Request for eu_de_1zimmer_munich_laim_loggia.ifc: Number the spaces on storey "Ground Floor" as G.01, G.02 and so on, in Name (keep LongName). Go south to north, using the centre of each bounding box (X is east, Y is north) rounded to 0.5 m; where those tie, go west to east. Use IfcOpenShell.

First a look at what the model holds.

```python
import ifcopenshell
import ifcopenshell.util.element
import ifcopenshell.util.placement

model = ifcopenshell.open("eu_de_1zimmer_munich_laim_loggia.ifc")
print(model.schema)
storey = next(s for s in model.by_type("IfcBuildingStorey") if s.Name == "Ground Floor")
spaces = [e for e in ifcopenshell.util.element.get_decomposition(storey) if e.is_a("IfcSpace")]
for e in sorted(spaces, key=lambda e: e.id()):
    origin = ifcopenshell.util.placement.get_local_placement(e.ObjectPlacement)[:3, 3]
    print(e.id(), e.Name, e.LongName, origin.round(2) + 0.0, sep=" | ")
```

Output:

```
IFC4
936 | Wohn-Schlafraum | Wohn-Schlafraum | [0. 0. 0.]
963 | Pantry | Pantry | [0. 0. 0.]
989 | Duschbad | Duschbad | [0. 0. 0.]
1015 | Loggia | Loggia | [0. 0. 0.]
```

```python
import ifcopenshell
import ifcopenshell.geom
import ifcopenshell.util.element
import ifcopenshell.util.shape

model = ifcopenshell.open("eu_de_1zimmer_munich_laim_loggia.ifc")
settings = ifcopenshell.geom.settings()
settings.set("use-world-coords", True)


def centre(element):
    shape = ifcopenshell.geom.create_shape(settings, element)
    return ifcopenshell.util.shape.get_bbox_centroid(shape.geometry)


storey = next(s for s in model.by_type("IfcBuildingStorey") if s.Name == "Ground Floor")
spaces = [e for e in ifcopenshell.util.element.get_decomposition(storey) if e.is_a("IfcSpace")]

# Insertion points can sit at a corner or the storey origin, so sort by the geometry (in metres).
centres = {e: centre(e) for e in spaces}
spaces.sort(key=lambda e: (round(centres[e][1] / 0.5), centres[e][0]))

for i, e in enumerate(spaces, start=1):
    number = f"G.{i:02d}"
    e.Name = number
    print(e.id(), number)

model.write("eu_de_1zimmer_munich_laim_loggia_rev.ifc")
```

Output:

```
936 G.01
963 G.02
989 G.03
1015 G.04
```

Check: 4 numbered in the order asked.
